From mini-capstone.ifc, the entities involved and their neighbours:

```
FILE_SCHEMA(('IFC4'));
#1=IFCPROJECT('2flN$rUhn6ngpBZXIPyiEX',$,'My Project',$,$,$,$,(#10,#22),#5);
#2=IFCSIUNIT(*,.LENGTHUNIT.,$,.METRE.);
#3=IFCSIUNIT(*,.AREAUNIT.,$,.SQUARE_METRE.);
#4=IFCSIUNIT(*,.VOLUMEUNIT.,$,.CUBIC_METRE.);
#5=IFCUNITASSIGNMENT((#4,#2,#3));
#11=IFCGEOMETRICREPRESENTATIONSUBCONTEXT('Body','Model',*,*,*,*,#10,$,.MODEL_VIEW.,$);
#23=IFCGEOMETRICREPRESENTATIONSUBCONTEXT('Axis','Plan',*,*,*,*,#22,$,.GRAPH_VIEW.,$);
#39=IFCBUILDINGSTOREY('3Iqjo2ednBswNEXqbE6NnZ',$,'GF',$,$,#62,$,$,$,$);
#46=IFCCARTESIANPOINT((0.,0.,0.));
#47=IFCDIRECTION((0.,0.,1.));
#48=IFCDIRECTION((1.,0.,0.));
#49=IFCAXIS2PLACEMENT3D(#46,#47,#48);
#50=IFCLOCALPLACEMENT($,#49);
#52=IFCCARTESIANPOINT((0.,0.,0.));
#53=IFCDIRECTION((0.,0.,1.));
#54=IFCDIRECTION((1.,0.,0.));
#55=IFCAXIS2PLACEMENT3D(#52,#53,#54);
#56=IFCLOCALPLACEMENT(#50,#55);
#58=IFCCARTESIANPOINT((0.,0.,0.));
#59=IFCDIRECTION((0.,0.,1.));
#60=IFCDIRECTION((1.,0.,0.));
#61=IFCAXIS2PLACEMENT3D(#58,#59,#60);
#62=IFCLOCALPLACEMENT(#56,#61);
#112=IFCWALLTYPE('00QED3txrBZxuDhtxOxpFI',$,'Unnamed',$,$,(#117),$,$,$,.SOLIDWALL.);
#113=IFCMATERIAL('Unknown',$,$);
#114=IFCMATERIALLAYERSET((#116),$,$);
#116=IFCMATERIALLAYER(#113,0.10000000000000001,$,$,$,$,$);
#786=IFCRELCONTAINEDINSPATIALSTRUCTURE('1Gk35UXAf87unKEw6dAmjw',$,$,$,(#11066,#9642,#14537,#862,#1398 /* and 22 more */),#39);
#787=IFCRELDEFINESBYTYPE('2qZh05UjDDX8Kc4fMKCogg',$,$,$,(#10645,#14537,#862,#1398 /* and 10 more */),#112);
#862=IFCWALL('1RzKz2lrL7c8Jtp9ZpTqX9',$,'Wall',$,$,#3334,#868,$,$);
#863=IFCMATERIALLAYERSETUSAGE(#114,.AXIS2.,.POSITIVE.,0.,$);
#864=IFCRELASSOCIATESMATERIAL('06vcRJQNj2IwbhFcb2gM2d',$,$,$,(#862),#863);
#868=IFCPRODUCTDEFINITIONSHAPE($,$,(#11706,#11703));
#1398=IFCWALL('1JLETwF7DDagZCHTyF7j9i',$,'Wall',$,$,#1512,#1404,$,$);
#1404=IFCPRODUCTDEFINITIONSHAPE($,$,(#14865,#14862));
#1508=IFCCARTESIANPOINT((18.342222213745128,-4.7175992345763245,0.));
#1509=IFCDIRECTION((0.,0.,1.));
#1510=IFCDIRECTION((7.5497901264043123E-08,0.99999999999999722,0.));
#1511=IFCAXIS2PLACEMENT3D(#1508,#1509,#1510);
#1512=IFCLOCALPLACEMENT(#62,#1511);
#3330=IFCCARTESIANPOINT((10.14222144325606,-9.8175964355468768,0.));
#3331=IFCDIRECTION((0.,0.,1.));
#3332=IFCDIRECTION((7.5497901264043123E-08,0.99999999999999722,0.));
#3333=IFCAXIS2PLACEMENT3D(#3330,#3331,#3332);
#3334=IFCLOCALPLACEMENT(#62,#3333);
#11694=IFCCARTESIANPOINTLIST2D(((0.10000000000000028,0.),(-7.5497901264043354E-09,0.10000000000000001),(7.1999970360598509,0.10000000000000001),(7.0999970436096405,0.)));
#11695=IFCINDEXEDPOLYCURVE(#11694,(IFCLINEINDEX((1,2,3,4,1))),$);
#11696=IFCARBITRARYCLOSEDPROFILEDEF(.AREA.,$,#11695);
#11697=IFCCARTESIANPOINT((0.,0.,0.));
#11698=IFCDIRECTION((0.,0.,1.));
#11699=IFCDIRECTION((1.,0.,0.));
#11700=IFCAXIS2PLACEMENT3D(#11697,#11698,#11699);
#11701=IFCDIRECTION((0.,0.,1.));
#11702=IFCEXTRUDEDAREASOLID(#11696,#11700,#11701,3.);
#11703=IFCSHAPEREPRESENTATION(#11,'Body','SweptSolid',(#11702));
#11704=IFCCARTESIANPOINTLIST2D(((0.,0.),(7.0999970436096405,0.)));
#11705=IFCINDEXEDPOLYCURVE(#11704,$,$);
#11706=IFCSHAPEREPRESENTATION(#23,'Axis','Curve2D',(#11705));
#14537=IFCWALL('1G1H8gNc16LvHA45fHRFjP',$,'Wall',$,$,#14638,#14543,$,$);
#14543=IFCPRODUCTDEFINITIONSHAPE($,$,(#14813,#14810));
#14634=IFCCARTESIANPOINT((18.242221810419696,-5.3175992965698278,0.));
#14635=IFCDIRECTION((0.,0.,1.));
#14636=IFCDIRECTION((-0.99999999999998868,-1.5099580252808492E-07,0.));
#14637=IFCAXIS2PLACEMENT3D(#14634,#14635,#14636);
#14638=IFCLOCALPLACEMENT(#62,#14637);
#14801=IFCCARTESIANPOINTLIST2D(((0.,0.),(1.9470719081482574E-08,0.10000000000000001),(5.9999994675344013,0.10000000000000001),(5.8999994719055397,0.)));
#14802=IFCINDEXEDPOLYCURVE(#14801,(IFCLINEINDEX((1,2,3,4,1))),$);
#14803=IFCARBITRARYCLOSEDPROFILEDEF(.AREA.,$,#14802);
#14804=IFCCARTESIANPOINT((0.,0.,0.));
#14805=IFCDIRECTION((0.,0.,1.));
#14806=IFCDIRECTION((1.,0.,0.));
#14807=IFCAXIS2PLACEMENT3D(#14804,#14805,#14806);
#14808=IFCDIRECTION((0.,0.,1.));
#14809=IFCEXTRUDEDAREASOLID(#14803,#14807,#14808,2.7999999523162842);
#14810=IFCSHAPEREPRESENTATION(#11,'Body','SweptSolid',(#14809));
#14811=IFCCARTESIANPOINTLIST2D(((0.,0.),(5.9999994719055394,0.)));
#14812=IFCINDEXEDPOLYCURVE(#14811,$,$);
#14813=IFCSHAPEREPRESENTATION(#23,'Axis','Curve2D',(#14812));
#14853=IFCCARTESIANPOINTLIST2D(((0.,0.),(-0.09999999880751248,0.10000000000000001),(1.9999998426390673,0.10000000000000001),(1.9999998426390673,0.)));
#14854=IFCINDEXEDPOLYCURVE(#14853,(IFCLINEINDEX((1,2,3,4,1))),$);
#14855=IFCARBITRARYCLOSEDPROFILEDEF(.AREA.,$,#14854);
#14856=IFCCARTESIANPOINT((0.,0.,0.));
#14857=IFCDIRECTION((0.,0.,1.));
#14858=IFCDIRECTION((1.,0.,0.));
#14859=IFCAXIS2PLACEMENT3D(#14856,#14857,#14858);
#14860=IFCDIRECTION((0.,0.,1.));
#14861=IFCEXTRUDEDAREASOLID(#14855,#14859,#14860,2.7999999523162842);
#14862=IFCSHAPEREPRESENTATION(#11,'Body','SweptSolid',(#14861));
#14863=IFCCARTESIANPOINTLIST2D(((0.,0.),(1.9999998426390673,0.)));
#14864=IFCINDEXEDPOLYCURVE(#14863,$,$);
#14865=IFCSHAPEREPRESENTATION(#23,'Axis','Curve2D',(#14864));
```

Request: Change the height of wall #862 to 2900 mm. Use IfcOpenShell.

```python
import ifcopenshell
import ifcopenshell.geom
import ifcopenshell.util.representation
import ifcopenshell.util.shape
import ifcopenshell.util.unit

model = ifcopenshell.open("mini-capstone.ifc")
unit_scale = ifcopenshell.util.unit.calculate_unit_scale(model)
settings = ifcopenshell.geom.settings()


def volume(element):
    """Net volume in cubic metres, openings subtracted."""
    shape = ifcopenshell.geom.create_shape(settings, element)
    return ifcopenshell.util.shape.get_volume(shape.geometry)


wall = model.by_id(862)
before = volume(wall)

body = ifcopenshell.util.representation.get_representation(wall, "Model", "Body")
solid = body.Items[0]
old_height = solid.Depth
solid.Depth = 2.9 / unit_scale
after = volume(wall)

print(f"height {old_height:g} -> {solid.Depth:g}, volume {before:.3f} -> {after:.3f} m3")

model.write("mini-capstone-out.ifc")
```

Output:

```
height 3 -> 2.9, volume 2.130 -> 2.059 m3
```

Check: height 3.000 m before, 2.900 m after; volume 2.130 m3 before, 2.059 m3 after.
